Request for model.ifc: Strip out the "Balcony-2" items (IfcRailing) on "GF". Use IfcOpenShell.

First a look at what the model holds.

```python
import ifcopenshell
import ifcopenshell.util.element

model = ifcopenshell.open("model.ifc")
print(model.schema)
storey = next(s for s in model.by_type("IfcBuildingStorey") if s.Name == "GF")
railings = [e for e in ifcopenshell.util.element.get_decomposition(storey) if e.is_a("IfcRailing")]
seen = {}
for e in railings:
    element_type = ifcopenshell.util.element.get_type(e)
    name = element_type.Name if element_type not in (None, e) else None
    seen[name] = seen.get(name, 0) + 1
for name, count in sorted(seen.items(), key=str):
    print(count, "x", name)
```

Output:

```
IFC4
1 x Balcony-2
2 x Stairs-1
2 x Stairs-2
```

```python
import ifcopenshell
import ifcopenshell.api.root
import ifcopenshell.util.element

model = ifcopenshell.open("model.ifc")

storey = next(s for s in model.by_type("IfcBuildingStorey") if s.Name == "GF")
railings = [e for e in ifcopenshell.util.element.get_decomposition(storey) if e.is_a("IfcRailing")]
targets = [e for e in railings if (t := ifcopenshell.util.element.get_type(e)) not in (None, e) and t.Name == "Balcony-2"]

for e in targets:
    ifcopenshell.api.root.remove_product(model, product=e)
print(len(targets), "removed")

model.write("model_v2.ifc")
```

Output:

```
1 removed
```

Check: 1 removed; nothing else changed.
